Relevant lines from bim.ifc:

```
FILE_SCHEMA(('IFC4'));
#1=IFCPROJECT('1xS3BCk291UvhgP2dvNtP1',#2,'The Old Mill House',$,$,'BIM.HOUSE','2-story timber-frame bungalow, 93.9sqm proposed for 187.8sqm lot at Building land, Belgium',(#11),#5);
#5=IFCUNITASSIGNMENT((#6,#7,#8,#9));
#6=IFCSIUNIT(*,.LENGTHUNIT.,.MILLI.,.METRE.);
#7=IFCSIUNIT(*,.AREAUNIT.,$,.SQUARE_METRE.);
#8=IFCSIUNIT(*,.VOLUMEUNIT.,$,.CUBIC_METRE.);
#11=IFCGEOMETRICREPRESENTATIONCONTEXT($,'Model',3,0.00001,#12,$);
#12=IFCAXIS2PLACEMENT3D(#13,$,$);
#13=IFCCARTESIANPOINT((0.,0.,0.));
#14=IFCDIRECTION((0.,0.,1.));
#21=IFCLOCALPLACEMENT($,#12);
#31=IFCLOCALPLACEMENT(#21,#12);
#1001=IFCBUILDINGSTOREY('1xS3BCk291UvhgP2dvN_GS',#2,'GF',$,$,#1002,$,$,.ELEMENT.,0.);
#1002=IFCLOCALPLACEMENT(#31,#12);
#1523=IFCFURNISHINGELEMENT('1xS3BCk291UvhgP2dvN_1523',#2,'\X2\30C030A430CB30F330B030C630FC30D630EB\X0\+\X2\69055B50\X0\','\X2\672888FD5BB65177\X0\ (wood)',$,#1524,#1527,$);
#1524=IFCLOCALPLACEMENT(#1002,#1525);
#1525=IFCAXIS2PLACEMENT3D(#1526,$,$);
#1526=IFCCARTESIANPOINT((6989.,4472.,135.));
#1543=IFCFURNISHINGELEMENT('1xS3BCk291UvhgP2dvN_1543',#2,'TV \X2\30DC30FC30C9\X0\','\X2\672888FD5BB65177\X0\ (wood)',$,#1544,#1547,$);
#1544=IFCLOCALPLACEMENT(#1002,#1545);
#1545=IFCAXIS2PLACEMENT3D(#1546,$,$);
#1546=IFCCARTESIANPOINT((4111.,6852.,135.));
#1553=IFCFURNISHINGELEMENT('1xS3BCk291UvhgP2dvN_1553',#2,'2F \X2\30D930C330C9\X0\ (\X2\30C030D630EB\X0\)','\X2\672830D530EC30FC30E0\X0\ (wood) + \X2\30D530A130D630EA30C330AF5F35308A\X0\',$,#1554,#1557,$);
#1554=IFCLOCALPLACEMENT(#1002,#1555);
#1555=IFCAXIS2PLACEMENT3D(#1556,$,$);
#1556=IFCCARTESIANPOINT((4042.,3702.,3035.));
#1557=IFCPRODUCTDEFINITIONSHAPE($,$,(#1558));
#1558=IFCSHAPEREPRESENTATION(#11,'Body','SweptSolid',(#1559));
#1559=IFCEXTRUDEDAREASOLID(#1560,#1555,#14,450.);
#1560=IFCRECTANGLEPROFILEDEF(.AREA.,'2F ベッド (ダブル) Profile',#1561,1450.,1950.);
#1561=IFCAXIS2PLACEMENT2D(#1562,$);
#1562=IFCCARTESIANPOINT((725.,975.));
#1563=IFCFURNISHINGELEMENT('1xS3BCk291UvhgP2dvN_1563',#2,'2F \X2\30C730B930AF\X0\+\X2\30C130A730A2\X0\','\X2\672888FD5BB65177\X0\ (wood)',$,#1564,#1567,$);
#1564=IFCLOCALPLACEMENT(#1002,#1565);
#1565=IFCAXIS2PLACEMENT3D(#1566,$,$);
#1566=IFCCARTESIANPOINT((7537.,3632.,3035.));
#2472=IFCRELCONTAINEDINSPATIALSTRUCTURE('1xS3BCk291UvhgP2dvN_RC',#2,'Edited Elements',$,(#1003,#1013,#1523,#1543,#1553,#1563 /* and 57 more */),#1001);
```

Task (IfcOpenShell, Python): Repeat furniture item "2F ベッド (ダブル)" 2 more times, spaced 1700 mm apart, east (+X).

```python
import numpy as np
import ifcopenshell
import ifcopenshell.api.geometry
import ifcopenshell.api.root
import ifcopenshell.util.element
import ifcopenshell.util.placement

model = ifcopenshell.open("bim.ifc")


def reuse_history(source, copy):
    """copy_class also copies each property set's owner history, people and application; keep the originals."""
    for rel in copy.IsDefinedBy:
        if rel.is_a("IfcRelDefinesByProperties") and (history := rel.RelatingPropertyDefinition.OwnerHistory):
            rel.RelatingPropertyDefinition.OwnerHistory = source.OwnerHistory
            ifcopenshell.util.element.remove_deep2(model, history)


source = model.by_id(1553)
base = ifcopenshell.util.placement.get_local_placement(source.ObjectPlacement)
step = np.array([1.0, 0.0, 0.0]) * 1700.0

for i in range(1, 3):
    copy = ifcopenshell.api.root.copy_class(model, product=source)
    copy.Representation = ifcopenshell.util.element.copy_deep(
        model, source.Representation, exclude=["IfcGeometricRepresentationContext", "IfcRepresentationMap"]
    )
    reuse_history(source, copy)
    matrix = base.copy()
    matrix[:3, 3] += i * step
    print("added at", matrix[:3, 3].round(3) + 0.0)
    ifcopenshell.api.geometry.edit_object_placement(model, product=copy, matrix=matrix, is_si=False)

model.write("bim_edited.ifc")
```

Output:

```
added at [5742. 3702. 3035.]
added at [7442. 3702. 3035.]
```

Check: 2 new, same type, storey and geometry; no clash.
